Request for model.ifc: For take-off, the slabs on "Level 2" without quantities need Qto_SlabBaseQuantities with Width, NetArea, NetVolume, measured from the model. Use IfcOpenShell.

First a look at what the model holds.

```python
import ifcopenshell
import ifcopenshell.util.element
import ifcopenshell.util.unit

model = ifcopenshell.open("model.ifc")
print(model.schema)
for unit_type in ("LENGTHUNIT", "AREAUNIT", "VOLUMEUNIT"):
    print(unit_type, ifcopenshell.util.unit.calculate_unit_scale(model, unit_type))
storey = next(s for s in model.by_type("IfcBuildingStorey") if s.Name == "Level 2")
slabs = [e for e in ifcopenshell.util.element.get_decomposition(storey) if e.is_a("IfcSlab")]
for e in sorted(slabs, key=lambda e: e.id()):
    print(e.id(), e.is_a(), e.Name, list(ifcopenshell.util.element.get_psets(e, qtos_only=True)), sep=" | ")
```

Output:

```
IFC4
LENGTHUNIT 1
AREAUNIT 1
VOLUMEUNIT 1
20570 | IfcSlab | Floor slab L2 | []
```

```python
import ifcopenshell
import ifcopenshell.api.pset
import ifcopenshell.geom
import ifcopenshell.util.element
import ifcopenshell.util.shape
import ifcopenshell.util.unit

model = ifcopenshell.open("model.ifc")
unit_scale = ifcopenshell.util.unit.calculate_unit_scale(model)
area_scale = ifcopenshell.util.unit.calculate_unit_scale(model, "AREAUNIT")
volume_scale = ifcopenshell.util.unit.calculate_unit_scale(model, "VOLUMEUNIT")
settings = ifcopenshell.geom.settings()

storey = next(s for s in model.by_type("IfcBuildingStorey") if s.Name == "Level 2")
slabs = [e for e in ifcopenshell.util.element.get_decomposition(storey) if e.is_a("IfcSlab")]

for e in sorted(slabs, key=lambda e: e.id()):
    if ifcopenshell.util.element.get_psets(e, qtos_only=True, should_inherit=False):
        continue
    # Geometry comes back in metres, in the element's own axes.
    shape = ifcopenshell.geom.create_shape(settings, e)
    values = {
        "Width": ifcopenshell.util.shape.get_z(shape.geometry) / unit_scale,
        "NetArea": ifcopenshell.util.shape.get_footprint_area(shape.geometry) / area_scale,
        "NetVolume": ifcopenshell.util.shape.get_volume(shape.geometry) / volume_scale,
    }
    qto = ifcopenshell.api.pset.add_qto(model, product=e, name="Qto_SlabBaseQuantities")
    ifcopenshell.api.pset.edit_qto(model, qto=qto, properties=values)
    print(e.id(), {k: round(v, 3) for k, v in values.items()})

model.write("model-out.ifc")
```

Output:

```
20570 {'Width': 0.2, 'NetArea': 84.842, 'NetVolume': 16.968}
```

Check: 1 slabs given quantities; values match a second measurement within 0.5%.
